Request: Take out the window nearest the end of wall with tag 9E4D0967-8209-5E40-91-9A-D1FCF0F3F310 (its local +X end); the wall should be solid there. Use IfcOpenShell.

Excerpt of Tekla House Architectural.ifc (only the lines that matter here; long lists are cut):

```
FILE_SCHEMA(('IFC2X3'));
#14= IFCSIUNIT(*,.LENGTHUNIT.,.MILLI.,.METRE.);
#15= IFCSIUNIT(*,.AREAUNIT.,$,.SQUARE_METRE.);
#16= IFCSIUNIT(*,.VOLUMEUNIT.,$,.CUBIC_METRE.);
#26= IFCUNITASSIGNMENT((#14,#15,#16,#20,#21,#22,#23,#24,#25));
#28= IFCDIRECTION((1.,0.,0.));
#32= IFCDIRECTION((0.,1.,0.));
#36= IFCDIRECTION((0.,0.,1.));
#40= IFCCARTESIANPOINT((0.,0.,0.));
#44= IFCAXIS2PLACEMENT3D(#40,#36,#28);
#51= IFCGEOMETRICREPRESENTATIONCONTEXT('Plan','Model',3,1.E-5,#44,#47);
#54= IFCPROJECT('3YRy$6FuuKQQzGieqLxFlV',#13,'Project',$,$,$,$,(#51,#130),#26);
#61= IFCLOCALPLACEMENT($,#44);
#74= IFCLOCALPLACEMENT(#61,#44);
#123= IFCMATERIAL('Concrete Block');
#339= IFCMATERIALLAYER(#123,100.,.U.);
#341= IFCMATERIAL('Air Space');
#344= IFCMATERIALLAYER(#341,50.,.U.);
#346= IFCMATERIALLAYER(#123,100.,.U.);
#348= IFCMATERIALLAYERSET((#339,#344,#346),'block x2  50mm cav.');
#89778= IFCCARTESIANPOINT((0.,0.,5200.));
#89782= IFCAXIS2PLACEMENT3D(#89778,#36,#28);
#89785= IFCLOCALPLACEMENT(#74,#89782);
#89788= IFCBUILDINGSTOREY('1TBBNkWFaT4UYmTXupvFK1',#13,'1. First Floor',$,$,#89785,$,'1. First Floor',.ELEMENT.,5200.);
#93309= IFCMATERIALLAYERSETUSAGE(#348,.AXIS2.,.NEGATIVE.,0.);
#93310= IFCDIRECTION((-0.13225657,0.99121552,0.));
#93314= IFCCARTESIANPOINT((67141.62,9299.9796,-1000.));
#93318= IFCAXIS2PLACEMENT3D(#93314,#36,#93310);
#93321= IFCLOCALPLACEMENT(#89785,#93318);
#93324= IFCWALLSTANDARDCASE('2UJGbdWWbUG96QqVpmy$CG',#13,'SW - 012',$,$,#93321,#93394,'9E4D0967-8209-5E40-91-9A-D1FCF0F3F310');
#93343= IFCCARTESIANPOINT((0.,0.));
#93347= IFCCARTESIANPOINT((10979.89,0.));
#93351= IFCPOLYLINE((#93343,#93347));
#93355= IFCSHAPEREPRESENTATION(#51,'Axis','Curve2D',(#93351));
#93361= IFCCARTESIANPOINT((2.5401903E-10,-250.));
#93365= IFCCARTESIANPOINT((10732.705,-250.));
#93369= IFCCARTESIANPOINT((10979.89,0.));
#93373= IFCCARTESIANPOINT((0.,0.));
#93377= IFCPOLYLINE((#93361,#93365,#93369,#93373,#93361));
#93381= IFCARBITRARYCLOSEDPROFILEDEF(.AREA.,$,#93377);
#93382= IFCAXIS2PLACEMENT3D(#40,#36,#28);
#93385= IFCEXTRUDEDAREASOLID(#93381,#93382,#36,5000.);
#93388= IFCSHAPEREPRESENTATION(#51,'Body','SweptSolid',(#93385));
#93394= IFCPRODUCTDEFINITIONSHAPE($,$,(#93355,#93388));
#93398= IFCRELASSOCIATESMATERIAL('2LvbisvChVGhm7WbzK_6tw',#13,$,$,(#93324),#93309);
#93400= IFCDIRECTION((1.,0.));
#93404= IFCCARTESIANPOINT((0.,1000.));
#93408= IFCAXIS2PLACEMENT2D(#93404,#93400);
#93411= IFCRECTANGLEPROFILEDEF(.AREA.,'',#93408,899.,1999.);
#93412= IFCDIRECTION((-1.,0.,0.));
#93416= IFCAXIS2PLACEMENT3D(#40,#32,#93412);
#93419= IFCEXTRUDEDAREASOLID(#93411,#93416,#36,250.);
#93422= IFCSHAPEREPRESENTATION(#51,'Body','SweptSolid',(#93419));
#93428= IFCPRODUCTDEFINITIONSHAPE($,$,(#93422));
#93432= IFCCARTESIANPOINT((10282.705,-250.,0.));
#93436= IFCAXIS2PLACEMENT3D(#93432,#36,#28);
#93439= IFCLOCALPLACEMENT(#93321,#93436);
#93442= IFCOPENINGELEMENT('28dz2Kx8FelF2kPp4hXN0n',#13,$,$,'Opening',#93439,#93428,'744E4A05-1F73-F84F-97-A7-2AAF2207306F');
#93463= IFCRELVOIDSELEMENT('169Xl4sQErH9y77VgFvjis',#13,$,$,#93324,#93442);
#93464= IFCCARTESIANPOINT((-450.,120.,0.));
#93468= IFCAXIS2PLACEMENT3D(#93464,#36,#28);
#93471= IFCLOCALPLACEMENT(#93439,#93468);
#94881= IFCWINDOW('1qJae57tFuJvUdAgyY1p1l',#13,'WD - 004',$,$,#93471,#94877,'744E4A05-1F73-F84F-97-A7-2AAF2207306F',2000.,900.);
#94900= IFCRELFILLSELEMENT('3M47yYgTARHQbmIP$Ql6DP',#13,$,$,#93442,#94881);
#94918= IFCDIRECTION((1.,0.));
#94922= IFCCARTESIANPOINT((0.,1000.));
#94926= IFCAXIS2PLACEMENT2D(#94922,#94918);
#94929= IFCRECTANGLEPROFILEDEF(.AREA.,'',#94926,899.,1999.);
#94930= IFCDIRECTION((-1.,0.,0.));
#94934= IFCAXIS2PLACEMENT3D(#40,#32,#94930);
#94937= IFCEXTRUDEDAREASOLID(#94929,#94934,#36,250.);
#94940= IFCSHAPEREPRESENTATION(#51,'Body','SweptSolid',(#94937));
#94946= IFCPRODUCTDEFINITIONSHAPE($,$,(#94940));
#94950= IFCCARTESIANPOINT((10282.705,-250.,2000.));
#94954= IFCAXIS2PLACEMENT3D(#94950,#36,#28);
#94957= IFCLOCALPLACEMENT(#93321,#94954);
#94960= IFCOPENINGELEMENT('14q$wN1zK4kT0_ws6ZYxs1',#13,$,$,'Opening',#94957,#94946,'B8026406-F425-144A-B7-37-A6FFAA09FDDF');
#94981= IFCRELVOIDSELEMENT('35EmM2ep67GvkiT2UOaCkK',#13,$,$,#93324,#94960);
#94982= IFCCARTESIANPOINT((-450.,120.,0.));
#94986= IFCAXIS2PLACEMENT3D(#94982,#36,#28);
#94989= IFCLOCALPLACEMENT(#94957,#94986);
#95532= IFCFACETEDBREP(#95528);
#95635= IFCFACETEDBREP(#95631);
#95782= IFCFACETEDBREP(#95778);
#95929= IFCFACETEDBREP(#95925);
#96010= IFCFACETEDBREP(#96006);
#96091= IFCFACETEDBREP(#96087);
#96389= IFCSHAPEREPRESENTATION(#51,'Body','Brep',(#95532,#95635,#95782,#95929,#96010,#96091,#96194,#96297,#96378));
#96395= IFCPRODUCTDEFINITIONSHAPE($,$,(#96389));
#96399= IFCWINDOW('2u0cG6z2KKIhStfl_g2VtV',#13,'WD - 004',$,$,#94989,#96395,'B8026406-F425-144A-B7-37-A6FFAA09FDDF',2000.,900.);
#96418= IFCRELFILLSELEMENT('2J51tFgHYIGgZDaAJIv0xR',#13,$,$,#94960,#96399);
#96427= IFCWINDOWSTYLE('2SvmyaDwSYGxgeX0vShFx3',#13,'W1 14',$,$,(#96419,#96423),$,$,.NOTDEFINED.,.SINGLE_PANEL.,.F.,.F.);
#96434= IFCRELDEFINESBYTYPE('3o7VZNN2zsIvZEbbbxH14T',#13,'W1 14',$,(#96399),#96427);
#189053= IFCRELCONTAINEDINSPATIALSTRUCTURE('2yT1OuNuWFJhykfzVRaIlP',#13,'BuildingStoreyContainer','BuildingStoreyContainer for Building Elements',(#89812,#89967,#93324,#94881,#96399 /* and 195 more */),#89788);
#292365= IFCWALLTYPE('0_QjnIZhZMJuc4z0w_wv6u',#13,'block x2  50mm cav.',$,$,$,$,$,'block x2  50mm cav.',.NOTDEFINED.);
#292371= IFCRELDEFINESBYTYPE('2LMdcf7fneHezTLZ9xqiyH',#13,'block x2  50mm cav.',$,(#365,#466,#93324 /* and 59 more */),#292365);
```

```python
import ifcopenshell
import ifcopenshell.api.feature
import ifcopenshell.api.root
import ifcopenshell.geom
import ifcopenshell.util.shape

model = ifcopenshell.open("Tekla House Architectural.ifc")
settings = ifcopenshell.geom.settings()


def volume(element):
    """Net volume in cubic metres, openings subtracted."""
    shape = ifcopenshell.geom.create_shape(settings, element)
    return ifcopenshell.util.shape.get_volume(shape.geometry)


window = model.by_guid("2u0cG6z2KKIhStfl_g2VtV")
opening = window.FillsVoids[0].RelatingOpeningElement
wall = opening.VoidsElements[0].RelatingBuildingElement
before = volume(wall)

ifcopenshell.api.root.remove_product(model, product=window)
ifcopenshell.api.feature.remove_feature(model, feature=opening)

after = volume(wall)

print(f"wall volume {before:.3f} -> {after:.3f} m3")

model.write("Tekla House Architectural-out.ifc")
```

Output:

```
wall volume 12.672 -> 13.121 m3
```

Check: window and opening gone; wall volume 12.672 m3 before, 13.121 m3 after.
